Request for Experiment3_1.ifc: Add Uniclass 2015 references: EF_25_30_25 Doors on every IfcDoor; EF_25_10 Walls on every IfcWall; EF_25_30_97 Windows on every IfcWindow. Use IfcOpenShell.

First a look at what the model holds.

```python
import ifcopenshell

model = ifcopenshell.open("Experiment3_1.ifc")
print(model.schema)
print("classifications:", [c.Name for c in model.by_type("IfcClassification")])
for ifc_class in ("IfcDoor", "IfcRoof", "IfcStair", "IfcWall", "IfcWindow"):
    print(ifc_class, len(model.by_type(ifc_class)))
```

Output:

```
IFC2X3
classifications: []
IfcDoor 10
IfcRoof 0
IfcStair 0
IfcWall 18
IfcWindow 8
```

```python
import ifcopenshell
import ifcopenshell.api.classification

model = ifcopenshell.open("Experiment3_1.ifc")

# IFC2X3 requires Source and Edition and has no link from the project to the system.
system = model.create_entity("IfcClassification", Source="NBS", Edition="2015", Name="Uniclass 2015")

codes = {
    "IfcDoor": ("EF_25_30_25", "Doors"),
    "IfcWall": ("EF_25_10", "Walls"),
    "IfcWindow": ("EF_25_30_97", "Windows"),
}
for ifc_class, (code, name) in codes.items():
    products = model.by_type(ifc_class)
    ifcopenshell.api.classification.add_reference(
        model, products=products, classification=system, identification=code, name=name
    )
    print(code, len(products))

model.write("Experiment3_1-out.ifc")
```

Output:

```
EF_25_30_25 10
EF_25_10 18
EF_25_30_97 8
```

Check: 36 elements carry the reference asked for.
